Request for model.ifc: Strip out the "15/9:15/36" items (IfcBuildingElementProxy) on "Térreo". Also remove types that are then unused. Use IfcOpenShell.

First a look at what the model holds.

```python
import ifcopenshell
import ifcopenshell.util.element

model = ifcopenshell.open("model.ifc")
print(model.schema)
storey = next(s for s in model.by_type("IfcBuildingStorey") if s.Name == "Térreo")
proxies = [e for e in ifcopenshell.util.element.get_decomposition(storey) if e.is_a("IfcBuildingElementProxy")]
seen = {}
for e in proxies:
    element_type = ifcopenshell.util.element.get_type(e)
    name = element_type.Name if element_type not in (None, e) else None
    seen[name] = seen.get(name, 0) + 1
for name, count in sorted(seen.items(), key=str):
    print(count, "x", name)
```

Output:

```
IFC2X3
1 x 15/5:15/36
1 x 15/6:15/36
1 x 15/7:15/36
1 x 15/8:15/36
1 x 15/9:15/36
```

```python
import ifcopenshell
import ifcopenshell.api.root
import ifcopenshell.util.element

model = ifcopenshell.open("model.ifc")

storey = next(s for s in model.by_type("IfcBuildingStorey") if s.Name == "Térreo")
proxies = [e for e in ifcopenshell.util.element.get_decomposition(storey) if e.is_a("IfcBuildingElementProxy")]
targets = [e for e in proxies if (t := ifcopenshell.util.element.get_type(e)) not in (None, e) and t.Name == "15/9:15/36"]
types = {ifcopenshell.util.element.get_type(e) for e in targets} - {None, *targets}

for e in targets:
    ifcopenshell.api.root.remove_product(model, product=e)
print(len(targets), "removed")

unused = [t for t in types if not ifcopenshell.util.element.get_types(t)]
for t in unused:
    ifcopenshell.api.root.remove_product(model, product=t)
print(len(unused), "unused types removed")

model.write("model-out.ifc")
```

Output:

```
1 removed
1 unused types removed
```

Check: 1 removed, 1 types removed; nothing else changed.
